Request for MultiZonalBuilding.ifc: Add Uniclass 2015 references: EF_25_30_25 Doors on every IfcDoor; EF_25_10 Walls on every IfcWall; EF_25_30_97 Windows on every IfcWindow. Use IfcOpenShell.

First a look at what the model holds.

```python
import ifcopenshell

model = ifcopenshell.open("MultiZonalBuilding.ifc")
print(model.schema)
print("classifications:", [c.Name for c in model.by_type("IfcClassification")])
for ifc_class in ("IfcDoor", "IfcRoof", "IfcStair", "IfcWall", "IfcWindow"):
    print(ifc_class, len(model.by_type(ifc_class)))
```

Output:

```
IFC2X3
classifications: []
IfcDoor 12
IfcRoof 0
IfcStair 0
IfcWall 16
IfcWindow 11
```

```python
import ifcopenshell
import ifcopenshell.api.classification

model = ifcopenshell.open("MultiZonalBuilding.ifc")

# IFC2X3 requires Source and Edition and has no link from the project to the system.
system = model.create_entity("IfcClassification", Source="NBS", Edition="2015", Name="Uniclass 2015")

codes = {
    "IfcDoor": ("EF_25_30_25", "Doors"),
    "IfcWall": ("EF_25_10", "Walls"),
    "IfcWindow": ("EF_25_30_97", "Windows"),
}
for ifc_class, (code, name) in codes.items():
    products = model.by_type(ifc_class)
    ifcopenshell.api.classification.add_reference(
        model, products=products, classification=system, identification=code, name=name
    )
    print(code, len(products))

model.write("MultiZonalBuilding_rev.ifc")
```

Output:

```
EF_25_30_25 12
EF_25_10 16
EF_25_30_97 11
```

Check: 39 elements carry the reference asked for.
